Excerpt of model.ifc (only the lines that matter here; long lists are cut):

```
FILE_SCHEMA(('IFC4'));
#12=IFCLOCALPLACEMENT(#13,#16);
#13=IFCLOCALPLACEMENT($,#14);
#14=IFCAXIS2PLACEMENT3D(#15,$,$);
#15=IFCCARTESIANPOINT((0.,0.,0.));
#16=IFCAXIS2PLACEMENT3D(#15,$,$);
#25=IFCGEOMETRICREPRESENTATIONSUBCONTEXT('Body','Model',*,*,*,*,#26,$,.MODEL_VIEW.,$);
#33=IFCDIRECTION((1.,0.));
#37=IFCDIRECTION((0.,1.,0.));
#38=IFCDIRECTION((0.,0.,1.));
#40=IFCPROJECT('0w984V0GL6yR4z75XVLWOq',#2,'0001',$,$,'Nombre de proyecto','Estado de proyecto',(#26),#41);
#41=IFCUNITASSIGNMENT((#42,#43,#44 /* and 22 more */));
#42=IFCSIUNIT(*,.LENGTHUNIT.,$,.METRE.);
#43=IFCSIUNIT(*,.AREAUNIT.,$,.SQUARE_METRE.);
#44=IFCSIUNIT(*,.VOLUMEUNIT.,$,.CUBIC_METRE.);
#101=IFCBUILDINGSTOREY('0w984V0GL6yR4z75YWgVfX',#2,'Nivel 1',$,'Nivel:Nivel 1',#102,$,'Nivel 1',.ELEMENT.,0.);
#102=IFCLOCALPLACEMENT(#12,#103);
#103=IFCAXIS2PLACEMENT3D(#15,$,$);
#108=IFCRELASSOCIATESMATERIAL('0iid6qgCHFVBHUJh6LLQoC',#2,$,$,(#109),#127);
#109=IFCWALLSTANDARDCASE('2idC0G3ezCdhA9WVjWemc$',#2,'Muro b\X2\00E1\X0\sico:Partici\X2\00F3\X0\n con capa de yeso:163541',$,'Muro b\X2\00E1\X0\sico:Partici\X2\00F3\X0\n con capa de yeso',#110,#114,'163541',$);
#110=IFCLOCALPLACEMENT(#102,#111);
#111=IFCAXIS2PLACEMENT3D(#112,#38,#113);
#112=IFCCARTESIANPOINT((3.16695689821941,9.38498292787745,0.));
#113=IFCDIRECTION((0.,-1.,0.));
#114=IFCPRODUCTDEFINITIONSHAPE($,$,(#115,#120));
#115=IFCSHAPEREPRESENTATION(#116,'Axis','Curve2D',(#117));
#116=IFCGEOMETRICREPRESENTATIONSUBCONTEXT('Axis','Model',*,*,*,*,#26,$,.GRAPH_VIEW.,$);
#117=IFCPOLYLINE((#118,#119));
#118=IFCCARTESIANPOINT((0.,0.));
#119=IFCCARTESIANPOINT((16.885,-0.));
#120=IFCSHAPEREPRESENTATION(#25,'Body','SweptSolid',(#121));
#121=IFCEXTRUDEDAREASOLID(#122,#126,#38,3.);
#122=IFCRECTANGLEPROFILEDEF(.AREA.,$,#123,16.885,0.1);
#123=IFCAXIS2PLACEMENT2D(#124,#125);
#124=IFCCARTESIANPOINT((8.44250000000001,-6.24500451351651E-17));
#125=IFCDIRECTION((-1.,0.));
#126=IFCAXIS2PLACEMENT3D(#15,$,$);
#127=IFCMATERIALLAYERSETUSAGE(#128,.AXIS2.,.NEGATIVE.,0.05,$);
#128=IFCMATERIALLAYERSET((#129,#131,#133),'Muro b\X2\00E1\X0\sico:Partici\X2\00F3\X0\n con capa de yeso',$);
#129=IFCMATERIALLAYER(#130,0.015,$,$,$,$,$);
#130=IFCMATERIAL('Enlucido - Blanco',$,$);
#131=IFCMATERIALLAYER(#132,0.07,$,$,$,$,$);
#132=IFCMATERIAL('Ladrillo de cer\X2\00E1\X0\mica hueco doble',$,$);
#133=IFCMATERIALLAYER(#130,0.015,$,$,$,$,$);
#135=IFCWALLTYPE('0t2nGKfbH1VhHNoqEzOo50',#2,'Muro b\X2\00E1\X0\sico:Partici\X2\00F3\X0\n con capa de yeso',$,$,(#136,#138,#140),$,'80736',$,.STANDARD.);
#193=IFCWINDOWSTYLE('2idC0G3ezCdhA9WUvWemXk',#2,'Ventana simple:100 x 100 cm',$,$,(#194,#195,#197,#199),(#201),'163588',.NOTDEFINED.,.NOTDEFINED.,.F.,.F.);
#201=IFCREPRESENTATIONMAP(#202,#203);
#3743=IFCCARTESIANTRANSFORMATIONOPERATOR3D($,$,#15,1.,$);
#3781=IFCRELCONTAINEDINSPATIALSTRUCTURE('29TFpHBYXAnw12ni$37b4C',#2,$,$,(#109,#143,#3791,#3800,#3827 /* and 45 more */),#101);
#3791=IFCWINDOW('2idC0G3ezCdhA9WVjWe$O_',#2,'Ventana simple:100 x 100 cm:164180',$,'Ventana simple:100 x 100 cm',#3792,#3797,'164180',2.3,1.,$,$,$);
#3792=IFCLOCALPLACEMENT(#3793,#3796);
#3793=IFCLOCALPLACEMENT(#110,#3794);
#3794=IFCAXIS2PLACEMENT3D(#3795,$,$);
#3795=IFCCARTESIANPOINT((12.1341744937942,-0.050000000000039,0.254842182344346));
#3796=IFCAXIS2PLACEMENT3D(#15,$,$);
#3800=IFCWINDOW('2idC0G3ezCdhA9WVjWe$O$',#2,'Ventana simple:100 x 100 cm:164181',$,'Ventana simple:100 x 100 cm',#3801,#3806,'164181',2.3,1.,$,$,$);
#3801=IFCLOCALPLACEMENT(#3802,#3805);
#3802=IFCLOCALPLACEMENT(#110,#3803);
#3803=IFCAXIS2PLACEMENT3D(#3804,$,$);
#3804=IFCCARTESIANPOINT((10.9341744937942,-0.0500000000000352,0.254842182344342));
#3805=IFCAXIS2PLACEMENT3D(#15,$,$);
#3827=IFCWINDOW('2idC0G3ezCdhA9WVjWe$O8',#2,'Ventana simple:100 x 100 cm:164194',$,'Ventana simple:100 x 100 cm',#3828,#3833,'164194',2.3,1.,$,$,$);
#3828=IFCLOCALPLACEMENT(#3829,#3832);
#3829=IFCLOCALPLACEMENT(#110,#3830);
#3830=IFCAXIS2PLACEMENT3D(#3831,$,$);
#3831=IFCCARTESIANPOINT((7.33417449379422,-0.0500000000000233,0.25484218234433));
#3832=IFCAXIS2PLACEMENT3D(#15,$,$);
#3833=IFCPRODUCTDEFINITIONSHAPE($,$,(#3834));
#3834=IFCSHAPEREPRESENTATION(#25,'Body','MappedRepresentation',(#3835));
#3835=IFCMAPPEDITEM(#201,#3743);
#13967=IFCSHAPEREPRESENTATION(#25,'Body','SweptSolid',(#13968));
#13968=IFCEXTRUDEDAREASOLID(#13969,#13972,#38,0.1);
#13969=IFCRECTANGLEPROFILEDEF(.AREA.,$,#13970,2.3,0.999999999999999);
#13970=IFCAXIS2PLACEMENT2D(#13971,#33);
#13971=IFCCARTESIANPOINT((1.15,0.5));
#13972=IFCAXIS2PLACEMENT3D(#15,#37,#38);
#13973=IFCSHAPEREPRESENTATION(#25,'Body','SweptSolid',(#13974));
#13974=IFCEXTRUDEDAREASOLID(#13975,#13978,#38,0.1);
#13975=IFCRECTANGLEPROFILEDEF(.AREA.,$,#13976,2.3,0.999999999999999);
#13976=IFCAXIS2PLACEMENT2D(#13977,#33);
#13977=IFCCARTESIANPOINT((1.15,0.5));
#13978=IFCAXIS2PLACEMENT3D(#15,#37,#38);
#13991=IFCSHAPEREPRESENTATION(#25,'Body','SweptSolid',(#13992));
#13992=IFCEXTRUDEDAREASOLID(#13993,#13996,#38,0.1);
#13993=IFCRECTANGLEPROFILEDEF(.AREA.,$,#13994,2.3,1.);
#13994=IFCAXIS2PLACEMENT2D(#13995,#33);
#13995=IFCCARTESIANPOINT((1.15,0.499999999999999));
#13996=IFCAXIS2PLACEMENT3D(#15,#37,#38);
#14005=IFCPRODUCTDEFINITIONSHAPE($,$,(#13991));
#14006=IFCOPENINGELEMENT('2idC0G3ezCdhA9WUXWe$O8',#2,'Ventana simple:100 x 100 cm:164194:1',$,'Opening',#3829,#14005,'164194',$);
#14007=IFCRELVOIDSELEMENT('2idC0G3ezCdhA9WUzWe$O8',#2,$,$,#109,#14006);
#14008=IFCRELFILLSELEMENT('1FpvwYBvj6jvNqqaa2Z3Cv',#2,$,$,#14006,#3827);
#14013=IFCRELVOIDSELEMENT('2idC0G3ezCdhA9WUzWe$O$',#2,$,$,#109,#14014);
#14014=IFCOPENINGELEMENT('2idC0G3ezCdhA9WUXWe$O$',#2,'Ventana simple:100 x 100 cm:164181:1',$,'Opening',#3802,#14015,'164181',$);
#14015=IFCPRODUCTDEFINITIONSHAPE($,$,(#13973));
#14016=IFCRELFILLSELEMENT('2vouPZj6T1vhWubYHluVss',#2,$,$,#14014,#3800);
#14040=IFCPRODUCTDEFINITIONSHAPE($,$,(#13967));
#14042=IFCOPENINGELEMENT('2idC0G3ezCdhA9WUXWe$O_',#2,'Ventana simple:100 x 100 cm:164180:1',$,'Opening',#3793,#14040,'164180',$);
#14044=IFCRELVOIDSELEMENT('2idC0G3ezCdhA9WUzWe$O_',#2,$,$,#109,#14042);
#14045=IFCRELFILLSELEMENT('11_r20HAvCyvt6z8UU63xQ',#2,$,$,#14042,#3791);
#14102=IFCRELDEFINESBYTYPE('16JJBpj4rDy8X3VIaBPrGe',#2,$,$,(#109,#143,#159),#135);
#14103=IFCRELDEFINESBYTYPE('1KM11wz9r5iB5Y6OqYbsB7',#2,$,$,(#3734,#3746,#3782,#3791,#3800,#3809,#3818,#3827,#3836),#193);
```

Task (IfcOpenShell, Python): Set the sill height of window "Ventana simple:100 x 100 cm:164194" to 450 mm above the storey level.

```python
import numpy as np
import ifcopenshell
import ifcopenshell.api.geometry
import ifcopenshell.geom
import ifcopenshell.util.element
import ifcopenshell.util.placement
import ifcopenshell.util.shape
import ifcopenshell.util.unit

model = ifcopenshell.open("model.ifc")
unit_scale = ifcopenshell.util.unit.calculate_unit_scale(model)

window = model.by_guid("2idC0G3ezCdhA9WVjWe$O8")
opening = window.FillsVoids[0].RelatingOpeningElement
storey = ifcopenshell.util.element.get_container(window, ifc_class="IfcBuildingStorey")
level = ifcopenshell.util.placement.get_local_placement(storey.ObjectPlacement)[2, 3]

# The opening's origin need not be at the sill, so measure its lowest point.
shape = ifcopenshell.geom.create_shape(ifcopenshell.geom.settings(), opening)
bottom = ifcopenshell.util.shape.get_shape_bottom_elevation(shape, shape.geometry) / unit_scale
dz = level + 0.45 / unit_scale - bottom

shift = np.array([0.0, 0.0, dz])
# The window is placed relative to its opening, so it follows when the opening moves.
matrix = ifcopenshell.util.placement.get_local_placement(opening.ObjectPlacement)
matrix[:3, 3] += shift
ifcopenshell.api.geometry.edit_object_placement(
    model, product=opening, matrix=matrix, is_si=False, should_transform_children=True
)

print(f"moved by {dz * unit_scale:+.3f} m")

model.write("model-out.ifc")
```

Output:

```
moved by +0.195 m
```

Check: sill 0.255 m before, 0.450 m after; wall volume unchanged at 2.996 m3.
